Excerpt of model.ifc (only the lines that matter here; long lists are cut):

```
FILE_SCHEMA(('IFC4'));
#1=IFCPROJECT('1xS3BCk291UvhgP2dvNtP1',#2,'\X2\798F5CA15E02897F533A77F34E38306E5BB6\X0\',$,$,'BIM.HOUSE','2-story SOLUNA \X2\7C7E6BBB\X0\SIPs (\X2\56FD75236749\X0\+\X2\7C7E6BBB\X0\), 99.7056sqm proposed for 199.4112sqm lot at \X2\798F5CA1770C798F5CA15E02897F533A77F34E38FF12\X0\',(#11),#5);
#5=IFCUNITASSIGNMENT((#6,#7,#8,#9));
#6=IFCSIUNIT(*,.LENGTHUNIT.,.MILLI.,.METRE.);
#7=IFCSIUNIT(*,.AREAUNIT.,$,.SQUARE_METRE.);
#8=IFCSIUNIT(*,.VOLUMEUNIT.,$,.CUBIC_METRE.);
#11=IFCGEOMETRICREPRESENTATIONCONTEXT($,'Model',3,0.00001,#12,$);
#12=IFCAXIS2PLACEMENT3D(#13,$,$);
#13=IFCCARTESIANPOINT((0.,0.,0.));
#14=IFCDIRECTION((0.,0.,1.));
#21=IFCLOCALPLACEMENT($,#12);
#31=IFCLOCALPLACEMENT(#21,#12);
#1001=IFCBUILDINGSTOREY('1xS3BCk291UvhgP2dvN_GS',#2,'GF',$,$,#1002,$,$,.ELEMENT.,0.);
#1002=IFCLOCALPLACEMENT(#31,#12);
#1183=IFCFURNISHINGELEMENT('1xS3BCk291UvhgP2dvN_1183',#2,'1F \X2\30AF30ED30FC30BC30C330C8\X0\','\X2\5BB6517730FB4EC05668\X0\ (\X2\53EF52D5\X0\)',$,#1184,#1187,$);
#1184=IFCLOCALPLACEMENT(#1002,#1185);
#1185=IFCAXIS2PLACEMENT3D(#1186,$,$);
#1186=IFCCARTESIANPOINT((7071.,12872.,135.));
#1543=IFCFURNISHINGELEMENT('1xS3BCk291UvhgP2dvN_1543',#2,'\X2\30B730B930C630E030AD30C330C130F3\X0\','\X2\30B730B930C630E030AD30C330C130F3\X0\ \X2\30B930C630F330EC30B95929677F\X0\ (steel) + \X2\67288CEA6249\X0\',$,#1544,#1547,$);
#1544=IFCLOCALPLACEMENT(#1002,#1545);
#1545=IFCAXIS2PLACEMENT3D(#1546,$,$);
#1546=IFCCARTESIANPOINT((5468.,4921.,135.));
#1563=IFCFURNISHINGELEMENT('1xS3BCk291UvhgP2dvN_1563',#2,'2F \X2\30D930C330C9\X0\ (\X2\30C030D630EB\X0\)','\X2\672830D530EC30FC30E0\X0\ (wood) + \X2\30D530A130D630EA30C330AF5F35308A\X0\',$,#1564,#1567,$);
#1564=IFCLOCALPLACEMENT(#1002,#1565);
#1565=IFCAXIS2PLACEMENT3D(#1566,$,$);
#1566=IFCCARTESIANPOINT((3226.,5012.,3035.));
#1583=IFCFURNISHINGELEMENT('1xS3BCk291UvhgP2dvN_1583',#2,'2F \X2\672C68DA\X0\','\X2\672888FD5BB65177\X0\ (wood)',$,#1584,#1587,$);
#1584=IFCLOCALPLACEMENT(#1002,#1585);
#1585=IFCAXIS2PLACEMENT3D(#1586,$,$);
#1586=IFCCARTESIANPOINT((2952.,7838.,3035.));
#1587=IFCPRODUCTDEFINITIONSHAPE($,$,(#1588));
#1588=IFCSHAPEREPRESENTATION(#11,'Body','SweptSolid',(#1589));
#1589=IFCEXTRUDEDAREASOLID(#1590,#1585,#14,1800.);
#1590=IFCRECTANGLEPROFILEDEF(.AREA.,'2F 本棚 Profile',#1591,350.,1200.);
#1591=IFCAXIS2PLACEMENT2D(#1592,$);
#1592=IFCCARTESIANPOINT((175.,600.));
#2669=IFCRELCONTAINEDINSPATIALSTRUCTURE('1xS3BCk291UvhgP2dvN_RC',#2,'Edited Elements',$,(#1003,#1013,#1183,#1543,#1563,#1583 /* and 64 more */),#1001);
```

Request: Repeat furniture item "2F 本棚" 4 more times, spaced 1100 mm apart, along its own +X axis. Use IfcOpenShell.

```python
import ifcopenshell
import ifcopenshell.api.geometry
import ifcopenshell.api.root
import ifcopenshell.util.element
import ifcopenshell.util.placement

model = ifcopenshell.open("model.ifc")


def reuse_history(source, copy):
    """copy_class also copies each property set's owner history, people and application; keep the originals."""
    for rel in copy.IsDefinedBy:
        if rel.is_a("IfcRelDefinesByProperties") and (history := rel.RelatingPropertyDefinition.OwnerHistory):
            rel.RelatingPropertyDefinition.OwnerHistory = source.OwnerHistory
            ifcopenshell.util.element.remove_deep2(model, history)


source = model.by_guid("1xS3BCk291UvhgP2dvN_1583")
base = ifcopenshell.util.placement.get_local_placement(source.ObjectPlacement)
step = base[:3, 0] * 1100.0

for i in range(1, 5):
    copy = ifcopenshell.api.root.copy_class(model, product=source)
    copy.Representation = ifcopenshell.util.element.copy_deep(
        model, source.Representation, exclude=["IfcGeometricRepresentationContext", "IfcRepresentationMap"]
    )
    reuse_history(source, copy)
    matrix = base.copy()
    matrix[:3, 3] += i * step
    print("added at", matrix[:3, 3].round(3) + 0.0)
    ifcopenshell.api.geometry.edit_object_placement(model, product=copy, matrix=matrix, is_si=False)

model.write("model-out.ifc")
```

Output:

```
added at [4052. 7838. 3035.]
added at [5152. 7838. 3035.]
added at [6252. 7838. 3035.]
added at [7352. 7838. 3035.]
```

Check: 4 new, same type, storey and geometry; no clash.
